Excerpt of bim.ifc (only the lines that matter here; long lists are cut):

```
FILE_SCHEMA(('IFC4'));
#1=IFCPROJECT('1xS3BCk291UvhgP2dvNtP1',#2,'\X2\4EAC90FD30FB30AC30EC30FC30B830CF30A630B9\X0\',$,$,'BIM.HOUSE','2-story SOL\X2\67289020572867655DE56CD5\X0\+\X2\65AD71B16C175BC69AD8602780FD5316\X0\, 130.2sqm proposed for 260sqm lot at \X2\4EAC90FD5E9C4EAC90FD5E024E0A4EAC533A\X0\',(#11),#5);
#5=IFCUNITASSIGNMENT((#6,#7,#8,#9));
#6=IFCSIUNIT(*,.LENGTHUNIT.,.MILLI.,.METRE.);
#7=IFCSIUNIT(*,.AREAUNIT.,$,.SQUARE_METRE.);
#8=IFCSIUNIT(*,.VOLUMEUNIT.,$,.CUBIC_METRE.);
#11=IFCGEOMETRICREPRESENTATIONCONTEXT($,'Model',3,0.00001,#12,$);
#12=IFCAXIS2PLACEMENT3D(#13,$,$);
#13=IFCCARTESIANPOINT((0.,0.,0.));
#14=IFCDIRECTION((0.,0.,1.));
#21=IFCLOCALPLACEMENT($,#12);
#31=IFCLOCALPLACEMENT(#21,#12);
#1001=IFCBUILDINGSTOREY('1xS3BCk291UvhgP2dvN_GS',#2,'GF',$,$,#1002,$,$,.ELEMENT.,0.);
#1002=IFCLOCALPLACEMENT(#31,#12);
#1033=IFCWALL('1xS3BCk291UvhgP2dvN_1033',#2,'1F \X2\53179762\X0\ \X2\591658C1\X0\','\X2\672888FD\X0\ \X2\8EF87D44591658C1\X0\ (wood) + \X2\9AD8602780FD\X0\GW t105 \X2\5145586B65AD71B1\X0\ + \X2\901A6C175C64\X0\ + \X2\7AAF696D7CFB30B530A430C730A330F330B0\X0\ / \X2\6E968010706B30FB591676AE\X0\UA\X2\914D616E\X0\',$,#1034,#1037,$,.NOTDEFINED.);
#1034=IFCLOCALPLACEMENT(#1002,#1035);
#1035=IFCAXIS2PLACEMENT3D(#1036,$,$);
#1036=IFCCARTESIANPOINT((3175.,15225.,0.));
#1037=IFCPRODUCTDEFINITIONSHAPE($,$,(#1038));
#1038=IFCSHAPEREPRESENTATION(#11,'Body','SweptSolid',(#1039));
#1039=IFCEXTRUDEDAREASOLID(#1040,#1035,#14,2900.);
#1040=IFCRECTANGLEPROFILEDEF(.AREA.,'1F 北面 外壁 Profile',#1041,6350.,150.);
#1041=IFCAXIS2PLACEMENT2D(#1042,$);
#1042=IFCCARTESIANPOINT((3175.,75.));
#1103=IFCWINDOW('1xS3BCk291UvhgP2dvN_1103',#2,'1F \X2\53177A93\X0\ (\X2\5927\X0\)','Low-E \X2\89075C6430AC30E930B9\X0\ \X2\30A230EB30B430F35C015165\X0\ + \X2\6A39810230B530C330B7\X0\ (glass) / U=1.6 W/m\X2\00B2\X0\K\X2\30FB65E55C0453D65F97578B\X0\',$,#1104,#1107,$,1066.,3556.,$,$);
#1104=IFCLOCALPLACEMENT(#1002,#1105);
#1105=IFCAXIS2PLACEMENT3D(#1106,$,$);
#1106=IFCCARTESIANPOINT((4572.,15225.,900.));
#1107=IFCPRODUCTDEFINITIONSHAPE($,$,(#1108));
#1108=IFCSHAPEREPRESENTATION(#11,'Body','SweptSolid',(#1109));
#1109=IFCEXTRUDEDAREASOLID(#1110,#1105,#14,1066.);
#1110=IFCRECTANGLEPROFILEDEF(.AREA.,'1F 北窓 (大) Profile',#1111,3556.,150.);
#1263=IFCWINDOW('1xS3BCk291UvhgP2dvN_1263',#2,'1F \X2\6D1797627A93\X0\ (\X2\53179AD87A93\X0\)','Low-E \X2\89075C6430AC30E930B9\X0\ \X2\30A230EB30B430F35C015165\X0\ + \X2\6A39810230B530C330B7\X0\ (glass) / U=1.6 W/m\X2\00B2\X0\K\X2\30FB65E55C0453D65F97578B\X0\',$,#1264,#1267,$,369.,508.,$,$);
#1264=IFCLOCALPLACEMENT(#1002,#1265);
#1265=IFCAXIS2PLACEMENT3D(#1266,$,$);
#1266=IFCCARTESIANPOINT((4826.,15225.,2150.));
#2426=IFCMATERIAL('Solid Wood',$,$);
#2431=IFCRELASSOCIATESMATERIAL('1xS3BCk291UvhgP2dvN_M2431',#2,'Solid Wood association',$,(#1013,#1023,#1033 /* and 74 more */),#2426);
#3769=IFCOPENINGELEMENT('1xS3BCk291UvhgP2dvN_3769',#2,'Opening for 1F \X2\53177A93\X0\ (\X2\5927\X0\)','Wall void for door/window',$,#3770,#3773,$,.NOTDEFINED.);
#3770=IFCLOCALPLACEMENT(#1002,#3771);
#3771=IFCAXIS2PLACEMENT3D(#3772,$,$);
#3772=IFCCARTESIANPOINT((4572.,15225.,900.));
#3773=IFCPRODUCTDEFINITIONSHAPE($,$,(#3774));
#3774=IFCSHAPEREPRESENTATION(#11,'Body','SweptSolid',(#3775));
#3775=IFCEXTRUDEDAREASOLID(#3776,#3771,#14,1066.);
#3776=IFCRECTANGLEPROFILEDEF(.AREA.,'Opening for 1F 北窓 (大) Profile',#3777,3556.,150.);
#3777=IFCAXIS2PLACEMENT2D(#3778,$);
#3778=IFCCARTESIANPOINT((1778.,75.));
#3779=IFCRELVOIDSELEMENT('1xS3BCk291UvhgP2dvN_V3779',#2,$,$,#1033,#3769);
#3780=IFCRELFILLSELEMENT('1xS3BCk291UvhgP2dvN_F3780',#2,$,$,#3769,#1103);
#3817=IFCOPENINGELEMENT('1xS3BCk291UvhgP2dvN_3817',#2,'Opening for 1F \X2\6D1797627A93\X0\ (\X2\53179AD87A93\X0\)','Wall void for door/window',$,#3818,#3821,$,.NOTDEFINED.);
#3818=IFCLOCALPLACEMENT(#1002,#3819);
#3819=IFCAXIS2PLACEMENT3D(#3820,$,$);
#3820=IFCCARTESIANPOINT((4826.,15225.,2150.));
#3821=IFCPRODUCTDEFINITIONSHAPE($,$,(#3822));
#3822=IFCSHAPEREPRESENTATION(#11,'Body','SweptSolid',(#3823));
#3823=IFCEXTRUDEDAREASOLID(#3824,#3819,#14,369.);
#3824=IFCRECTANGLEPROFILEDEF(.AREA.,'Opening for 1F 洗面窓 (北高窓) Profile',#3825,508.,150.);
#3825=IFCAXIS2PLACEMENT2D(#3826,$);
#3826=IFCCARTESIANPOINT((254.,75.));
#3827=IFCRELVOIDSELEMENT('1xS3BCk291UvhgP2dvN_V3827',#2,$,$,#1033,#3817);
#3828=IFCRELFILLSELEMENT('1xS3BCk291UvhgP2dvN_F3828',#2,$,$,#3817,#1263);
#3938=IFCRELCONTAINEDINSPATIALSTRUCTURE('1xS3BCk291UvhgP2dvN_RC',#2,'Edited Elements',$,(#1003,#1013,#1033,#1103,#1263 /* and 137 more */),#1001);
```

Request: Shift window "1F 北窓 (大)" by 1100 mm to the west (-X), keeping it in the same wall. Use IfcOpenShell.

```python
import ifcopenshell
import ifcopenshell.api.geometry
import ifcopenshell.util.placement
import ifcopenshell.util.unit

model = ifcopenshell.open("bim.ifc")
unit_scale = ifcopenshell.util.unit.calculate_unit_scale(model)

window = model.by_guid("1xS3BCk291UvhgP2dvN_1103")
opening = window.FillsVoids[0].RelatingOpeningElement
wall = opening.VoidsElements[0].RelatingBuildingElement

wall_matrix = ifcopenshell.util.placement.get_local_placement(wall.ObjectPlacement)
shift = wall_matrix[:3, 0] * -1.1 / unit_scale
before = ifcopenshell.util.placement.get_local_placement(window.ObjectPlacement)[:3, 3].copy()

# The window is not placed relative to its opening, so move both.
for product in (opening, window):
    matrix = ifcopenshell.util.placement.get_local_placement(product.ObjectPlacement)
    matrix[:3, 3] += shift
    ifcopenshell.api.geometry.edit_object_placement(model, product=product, matrix=matrix, is_si=False)

after = ifcopenshell.util.placement.get_local_placement(window.ObjectPlacement)[:3, 3]
print("window moved by", (after - before).round(3) + 0.0)

model.write("bim_rev.ifc")
```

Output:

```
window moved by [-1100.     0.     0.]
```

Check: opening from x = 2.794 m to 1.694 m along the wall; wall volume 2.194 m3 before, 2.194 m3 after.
